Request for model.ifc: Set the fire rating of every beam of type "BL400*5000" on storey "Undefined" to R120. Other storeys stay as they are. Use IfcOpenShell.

First a look at what the model holds.

```python
import ifcopenshell
import ifcopenshell.util.element

model = ifcopenshell.open("model.ifc")
print(model.schema)
storey = next(s for s in model.by_type("IfcBuildingStorey") if s.Name == "Undefined")
beams = [e for e in ifcopenshell.util.element.get_decomposition(storey) if e.is_a("IfcBeam")]
seen = {}
for e in beams:
    element_type = ifcopenshell.util.element.get_type(e)
    key = (element_type.Name if element_type != e and element_type else None, ifcopenshell.util.element.get_pset(e, "Pset_BeamCommon", "FireRating"))
    seen[key] = seen.get(key, 0) + 1
for (name, value), count in sorted(seen.items(), key=str):
    print(count, "x", name, "|", value)
```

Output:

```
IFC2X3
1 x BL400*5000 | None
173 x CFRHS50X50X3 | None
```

```python
import ifcopenshell
import ifcopenshell.api.pset
import ifcopenshell.util.element

model = ifcopenshell.open("model.ifc")

storey = next(s for s in model.by_type("IfcBuildingStorey") if s.Name == "Undefined")
beams = [e for e in ifcopenshell.util.element.get_decomposition(storey) if e.is_a("IfcBeam")]

count = 0
for e in beams:
    element_type = ifcopenshell.util.element.get_type(e)
    if element_type in (None, e) or element_type.Name != "BL400*5000":
        continue
    # add_pset returns the element's existing set when there is one.
    pset = ifcopenshell.api.pset.add_pset(model, product=e, name="Pset_BeamCommon")
    ifcopenshell.api.pset.edit_pset(model, pset=pset, properties={"FireRating": "R120"})
    count += 1

print(count, "beams updated")

model.write("model_rev.ifc")
```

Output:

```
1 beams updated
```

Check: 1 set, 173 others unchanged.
